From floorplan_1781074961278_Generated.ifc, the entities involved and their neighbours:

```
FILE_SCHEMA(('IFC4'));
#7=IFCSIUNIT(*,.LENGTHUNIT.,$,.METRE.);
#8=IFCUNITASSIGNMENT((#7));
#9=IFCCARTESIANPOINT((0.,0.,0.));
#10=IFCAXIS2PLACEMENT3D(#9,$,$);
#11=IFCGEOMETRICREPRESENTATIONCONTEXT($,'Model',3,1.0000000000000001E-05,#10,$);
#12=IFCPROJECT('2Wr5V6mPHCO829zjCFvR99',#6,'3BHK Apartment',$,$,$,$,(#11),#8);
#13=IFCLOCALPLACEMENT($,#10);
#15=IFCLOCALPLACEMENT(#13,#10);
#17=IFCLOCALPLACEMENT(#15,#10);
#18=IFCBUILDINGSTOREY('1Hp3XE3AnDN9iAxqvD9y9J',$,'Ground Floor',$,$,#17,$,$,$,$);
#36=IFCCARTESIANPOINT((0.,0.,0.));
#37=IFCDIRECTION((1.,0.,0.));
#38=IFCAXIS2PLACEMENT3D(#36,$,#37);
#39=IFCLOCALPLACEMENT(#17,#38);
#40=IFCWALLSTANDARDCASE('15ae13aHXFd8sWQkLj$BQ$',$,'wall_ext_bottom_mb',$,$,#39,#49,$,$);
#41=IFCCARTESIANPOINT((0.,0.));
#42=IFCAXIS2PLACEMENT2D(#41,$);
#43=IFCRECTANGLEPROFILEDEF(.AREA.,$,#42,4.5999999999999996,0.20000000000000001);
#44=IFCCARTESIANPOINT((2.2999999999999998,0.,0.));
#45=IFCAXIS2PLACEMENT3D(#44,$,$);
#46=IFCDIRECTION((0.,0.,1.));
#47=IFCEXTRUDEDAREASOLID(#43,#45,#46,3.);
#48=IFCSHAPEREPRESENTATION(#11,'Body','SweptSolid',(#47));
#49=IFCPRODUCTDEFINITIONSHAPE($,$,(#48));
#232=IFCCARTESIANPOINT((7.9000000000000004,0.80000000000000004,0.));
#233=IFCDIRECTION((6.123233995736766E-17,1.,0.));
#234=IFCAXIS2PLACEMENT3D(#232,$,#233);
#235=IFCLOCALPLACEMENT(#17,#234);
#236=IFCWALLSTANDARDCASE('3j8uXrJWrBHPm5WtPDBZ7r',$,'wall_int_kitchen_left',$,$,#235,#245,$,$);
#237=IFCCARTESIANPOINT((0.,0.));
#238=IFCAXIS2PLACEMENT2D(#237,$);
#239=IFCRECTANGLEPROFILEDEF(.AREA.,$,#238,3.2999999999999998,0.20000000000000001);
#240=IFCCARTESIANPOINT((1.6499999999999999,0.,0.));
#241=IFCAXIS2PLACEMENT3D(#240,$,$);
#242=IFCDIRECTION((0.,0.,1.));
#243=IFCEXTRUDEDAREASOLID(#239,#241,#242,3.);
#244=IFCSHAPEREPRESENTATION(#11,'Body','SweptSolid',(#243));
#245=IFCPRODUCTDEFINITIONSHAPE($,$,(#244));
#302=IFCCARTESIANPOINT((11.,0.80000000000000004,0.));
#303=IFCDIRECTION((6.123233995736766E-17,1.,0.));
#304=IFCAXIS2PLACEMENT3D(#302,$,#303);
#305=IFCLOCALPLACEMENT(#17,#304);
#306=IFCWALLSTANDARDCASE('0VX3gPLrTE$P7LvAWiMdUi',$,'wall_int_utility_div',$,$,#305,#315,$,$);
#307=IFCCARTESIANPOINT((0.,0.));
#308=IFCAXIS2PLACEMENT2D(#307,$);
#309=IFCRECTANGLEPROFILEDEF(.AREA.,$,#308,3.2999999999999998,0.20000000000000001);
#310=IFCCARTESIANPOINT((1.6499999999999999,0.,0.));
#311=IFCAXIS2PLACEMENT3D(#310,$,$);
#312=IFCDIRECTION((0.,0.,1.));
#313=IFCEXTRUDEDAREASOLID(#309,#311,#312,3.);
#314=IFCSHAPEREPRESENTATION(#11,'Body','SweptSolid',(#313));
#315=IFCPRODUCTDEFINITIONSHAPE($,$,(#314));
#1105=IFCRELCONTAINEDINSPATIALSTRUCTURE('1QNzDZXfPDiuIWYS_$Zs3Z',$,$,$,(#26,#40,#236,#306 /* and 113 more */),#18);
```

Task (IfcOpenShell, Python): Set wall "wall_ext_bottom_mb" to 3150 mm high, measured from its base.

```python
import ifcopenshell
import ifcopenshell.geom
import ifcopenshell.util.shape
import ifcopenshell.util.unit

model = ifcopenshell.open("floorplan_1781074961278_Generated.ifc")
unit_scale = ifcopenshell.util.unit.calculate_unit_scale(model)
settings = ifcopenshell.geom.settings()


def volume(element):
    """Net volume in cubic metres, openings subtracted."""
    shape = ifcopenshell.geom.create_shape(settings, element)
    return ifcopenshell.util.shape.get_volume(shape.geometry)


wall = model.by_guid("15ae13aHXFd8sWQkLj$BQ$")
before = volume(wall)

body = next(r for r in wall.Representation.Representations if r.RepresentationIdentifier == "Body")
solid = body.Items[0]
old_height = solid.Depth
solid.Depth = 3.15 / unit_scale
after = volume(wall)

print(f"height {old_height:g} -> {solid.Depth:g}, volume {before:.3f} -> {after:.3f} m3")

model.write("floorplan_1781074961278_Generated-out.ifc")
```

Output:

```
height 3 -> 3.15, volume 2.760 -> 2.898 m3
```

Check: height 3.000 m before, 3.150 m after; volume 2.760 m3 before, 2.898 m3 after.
